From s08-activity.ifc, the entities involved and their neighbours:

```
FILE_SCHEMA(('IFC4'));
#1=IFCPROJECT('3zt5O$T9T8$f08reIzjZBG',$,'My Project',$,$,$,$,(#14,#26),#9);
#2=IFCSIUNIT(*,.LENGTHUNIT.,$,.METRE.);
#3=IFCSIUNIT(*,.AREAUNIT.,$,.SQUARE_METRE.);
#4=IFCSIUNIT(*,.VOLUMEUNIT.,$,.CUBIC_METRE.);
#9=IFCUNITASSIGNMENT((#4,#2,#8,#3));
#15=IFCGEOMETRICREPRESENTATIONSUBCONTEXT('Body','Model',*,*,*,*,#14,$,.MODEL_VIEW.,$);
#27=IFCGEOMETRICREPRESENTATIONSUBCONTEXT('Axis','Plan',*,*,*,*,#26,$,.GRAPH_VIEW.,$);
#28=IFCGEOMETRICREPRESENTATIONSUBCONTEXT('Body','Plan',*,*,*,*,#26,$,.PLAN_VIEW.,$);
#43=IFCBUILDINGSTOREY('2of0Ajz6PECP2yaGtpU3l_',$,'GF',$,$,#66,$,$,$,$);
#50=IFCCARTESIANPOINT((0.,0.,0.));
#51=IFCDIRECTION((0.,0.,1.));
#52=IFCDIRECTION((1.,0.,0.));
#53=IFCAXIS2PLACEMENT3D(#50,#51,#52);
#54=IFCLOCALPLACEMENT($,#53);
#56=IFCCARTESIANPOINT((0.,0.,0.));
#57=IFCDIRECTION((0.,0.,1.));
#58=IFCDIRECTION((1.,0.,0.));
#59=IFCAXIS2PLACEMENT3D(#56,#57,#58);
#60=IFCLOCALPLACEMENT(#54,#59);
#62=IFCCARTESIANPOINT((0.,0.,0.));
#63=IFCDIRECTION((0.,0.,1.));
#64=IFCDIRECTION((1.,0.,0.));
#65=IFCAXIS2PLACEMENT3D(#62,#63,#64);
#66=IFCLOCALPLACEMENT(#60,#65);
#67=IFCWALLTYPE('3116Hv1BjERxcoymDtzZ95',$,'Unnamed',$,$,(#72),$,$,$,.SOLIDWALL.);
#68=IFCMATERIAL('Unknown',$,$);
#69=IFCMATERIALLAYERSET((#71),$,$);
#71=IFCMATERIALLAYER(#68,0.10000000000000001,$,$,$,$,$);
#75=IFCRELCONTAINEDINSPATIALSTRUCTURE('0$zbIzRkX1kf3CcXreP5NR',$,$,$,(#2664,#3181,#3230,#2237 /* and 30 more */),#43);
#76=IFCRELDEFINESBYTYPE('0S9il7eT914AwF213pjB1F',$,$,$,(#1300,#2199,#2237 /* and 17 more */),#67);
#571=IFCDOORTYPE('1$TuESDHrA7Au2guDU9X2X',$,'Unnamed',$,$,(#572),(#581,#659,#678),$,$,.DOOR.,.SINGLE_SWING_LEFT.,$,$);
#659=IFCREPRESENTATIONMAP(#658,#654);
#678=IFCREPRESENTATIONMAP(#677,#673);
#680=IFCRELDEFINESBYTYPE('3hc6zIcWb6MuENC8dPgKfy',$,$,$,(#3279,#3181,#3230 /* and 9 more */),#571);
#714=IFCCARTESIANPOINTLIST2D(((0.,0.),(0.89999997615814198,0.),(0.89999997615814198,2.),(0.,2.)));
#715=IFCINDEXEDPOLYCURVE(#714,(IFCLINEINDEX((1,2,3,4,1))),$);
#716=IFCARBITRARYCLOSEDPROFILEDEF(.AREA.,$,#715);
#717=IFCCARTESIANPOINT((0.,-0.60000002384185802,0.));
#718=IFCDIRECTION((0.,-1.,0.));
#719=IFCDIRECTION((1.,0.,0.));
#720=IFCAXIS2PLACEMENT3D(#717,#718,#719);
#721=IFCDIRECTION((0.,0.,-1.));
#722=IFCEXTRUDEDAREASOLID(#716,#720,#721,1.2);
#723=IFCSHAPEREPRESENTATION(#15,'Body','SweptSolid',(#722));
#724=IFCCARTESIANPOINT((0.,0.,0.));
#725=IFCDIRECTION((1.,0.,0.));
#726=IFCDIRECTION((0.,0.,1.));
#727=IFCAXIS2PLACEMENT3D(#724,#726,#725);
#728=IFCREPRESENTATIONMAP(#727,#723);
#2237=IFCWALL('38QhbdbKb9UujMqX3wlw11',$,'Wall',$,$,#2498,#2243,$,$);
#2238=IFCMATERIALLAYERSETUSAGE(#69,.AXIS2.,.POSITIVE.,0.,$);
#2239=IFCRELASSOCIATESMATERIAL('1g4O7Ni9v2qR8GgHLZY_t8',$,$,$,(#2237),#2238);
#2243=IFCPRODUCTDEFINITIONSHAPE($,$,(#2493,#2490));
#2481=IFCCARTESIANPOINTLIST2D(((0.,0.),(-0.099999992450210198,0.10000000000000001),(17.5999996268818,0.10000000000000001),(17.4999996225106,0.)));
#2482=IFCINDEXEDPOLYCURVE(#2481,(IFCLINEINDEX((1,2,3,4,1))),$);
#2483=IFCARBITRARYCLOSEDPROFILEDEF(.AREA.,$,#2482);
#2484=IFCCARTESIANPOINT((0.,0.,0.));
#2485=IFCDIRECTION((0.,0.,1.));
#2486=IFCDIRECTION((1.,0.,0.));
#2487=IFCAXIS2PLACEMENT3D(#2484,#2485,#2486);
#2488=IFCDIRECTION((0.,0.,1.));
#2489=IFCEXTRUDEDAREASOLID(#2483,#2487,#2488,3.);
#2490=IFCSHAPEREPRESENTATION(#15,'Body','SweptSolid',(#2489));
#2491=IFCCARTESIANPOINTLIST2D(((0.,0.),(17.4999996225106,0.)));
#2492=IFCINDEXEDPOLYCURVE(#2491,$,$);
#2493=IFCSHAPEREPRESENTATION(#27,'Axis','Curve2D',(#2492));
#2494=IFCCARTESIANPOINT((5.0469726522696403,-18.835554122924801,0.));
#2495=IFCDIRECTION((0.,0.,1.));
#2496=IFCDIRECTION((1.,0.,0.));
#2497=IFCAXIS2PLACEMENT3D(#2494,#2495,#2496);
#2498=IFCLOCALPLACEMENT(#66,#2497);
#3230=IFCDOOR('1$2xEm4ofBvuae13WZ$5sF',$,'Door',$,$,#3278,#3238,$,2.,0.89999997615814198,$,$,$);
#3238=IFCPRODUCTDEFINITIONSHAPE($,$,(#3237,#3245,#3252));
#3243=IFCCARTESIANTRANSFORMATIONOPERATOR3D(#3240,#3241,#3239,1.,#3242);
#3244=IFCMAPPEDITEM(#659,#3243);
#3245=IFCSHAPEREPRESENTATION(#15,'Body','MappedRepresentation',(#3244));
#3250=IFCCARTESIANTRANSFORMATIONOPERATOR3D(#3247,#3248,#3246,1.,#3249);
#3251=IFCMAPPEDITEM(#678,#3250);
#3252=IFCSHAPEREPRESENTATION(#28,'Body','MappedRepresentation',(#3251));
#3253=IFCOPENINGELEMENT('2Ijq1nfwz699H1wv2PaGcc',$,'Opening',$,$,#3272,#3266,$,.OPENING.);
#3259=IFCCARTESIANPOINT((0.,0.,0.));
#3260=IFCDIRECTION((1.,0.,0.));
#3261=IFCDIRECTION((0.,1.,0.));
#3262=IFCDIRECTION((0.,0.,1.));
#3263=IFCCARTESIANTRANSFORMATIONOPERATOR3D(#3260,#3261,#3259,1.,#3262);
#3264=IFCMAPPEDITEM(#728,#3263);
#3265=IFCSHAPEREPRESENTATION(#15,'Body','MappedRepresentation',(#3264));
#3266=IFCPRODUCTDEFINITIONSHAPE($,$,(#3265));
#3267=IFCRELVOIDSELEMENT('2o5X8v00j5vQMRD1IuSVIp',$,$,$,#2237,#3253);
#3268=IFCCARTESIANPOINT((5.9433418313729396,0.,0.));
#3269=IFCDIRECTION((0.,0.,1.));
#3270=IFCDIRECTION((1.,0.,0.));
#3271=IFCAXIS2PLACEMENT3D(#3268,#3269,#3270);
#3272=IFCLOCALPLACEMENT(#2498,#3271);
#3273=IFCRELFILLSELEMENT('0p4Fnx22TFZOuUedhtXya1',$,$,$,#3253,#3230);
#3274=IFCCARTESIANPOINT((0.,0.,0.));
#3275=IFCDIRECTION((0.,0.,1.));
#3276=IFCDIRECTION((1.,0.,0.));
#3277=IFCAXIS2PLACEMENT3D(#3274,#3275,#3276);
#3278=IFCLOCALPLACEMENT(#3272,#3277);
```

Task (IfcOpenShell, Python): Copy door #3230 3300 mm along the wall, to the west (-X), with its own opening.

```python
import ifcopenshell
import ifcopenshell.api.feature
import ifcopenshell.api.geometry
import ifcopenshell.api.root
import ifcopenshell.geom
import ifcopenshell.util.element
import ifcopenshell.util.placement
import ifcopenshell.util.shape
import ifcopenshell.util.unit

model = ifcopenshell.open("s08-activity.ifc")
unit_scale = ifcopenshell.util.unit.calculate_unit_scale(model)
settings = ifcopenshell.geom.settings()


def volume(element):
    """Net volume in cubic metres, openings subtracted."""
    shape = ifcopenshell.geom.create_shape(settings, element)
    return ifcopenshell.util.shape.get_volume(shape.geometry)


door = model.by_guid("1$2xEm4ofBvuae13WZ$5sF")
opening = door.FillsVoids[0].RelatingOpeningElement
wall = opening.VoidsElements[0].RelatingBuildingElement
before = volume(wall)
shift = ifcopenshell.util.placement.get_local_placement(wall.ObjectPlacement)[:3, 0] * -3.3 / unit_scale

# copy_class copies the void relationship, type, container and properties, but no geometry.
new_opening = ifcopenshell.api.root.copy_class(model, product=opening)
new_opening.Representation = ifcopenshell.util.element.copy_deep(
    model, opening.Representation, exclude=["IfcGeometricRepresentationContext", "IfcRepresentationMap"]
)
new_door = ifcopenshell.api.root.copy_class(model, product=door)
new_door.Representation = ifcopenshell.util.element.copy_deep(
    model, door.Representation, exclude=["IfcGeometricRepresentationContext", "IfcRepresentationMap"]
)
ifcopenshell.api.feature.add_filling(model, opening=new_opening, element=new_door)

for old, new in ((opening, new_opening), (door, new_door)):
    matrix = ifcopenshell.util.placement.get_local_placement(old.ObjectPlacement)
    matrix[:3, 3] += shift
    ifcopenshell.api.geometry.edit_object_placement(model, product=new, matrix=matrix, is_si=False)

after = volume(wall)

print(f"wall volume {before:.3f} -> {after:.3f} m3")

model.write("s08-activity-out.ifc")
```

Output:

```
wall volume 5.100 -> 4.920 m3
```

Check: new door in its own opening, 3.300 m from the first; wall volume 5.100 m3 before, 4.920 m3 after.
